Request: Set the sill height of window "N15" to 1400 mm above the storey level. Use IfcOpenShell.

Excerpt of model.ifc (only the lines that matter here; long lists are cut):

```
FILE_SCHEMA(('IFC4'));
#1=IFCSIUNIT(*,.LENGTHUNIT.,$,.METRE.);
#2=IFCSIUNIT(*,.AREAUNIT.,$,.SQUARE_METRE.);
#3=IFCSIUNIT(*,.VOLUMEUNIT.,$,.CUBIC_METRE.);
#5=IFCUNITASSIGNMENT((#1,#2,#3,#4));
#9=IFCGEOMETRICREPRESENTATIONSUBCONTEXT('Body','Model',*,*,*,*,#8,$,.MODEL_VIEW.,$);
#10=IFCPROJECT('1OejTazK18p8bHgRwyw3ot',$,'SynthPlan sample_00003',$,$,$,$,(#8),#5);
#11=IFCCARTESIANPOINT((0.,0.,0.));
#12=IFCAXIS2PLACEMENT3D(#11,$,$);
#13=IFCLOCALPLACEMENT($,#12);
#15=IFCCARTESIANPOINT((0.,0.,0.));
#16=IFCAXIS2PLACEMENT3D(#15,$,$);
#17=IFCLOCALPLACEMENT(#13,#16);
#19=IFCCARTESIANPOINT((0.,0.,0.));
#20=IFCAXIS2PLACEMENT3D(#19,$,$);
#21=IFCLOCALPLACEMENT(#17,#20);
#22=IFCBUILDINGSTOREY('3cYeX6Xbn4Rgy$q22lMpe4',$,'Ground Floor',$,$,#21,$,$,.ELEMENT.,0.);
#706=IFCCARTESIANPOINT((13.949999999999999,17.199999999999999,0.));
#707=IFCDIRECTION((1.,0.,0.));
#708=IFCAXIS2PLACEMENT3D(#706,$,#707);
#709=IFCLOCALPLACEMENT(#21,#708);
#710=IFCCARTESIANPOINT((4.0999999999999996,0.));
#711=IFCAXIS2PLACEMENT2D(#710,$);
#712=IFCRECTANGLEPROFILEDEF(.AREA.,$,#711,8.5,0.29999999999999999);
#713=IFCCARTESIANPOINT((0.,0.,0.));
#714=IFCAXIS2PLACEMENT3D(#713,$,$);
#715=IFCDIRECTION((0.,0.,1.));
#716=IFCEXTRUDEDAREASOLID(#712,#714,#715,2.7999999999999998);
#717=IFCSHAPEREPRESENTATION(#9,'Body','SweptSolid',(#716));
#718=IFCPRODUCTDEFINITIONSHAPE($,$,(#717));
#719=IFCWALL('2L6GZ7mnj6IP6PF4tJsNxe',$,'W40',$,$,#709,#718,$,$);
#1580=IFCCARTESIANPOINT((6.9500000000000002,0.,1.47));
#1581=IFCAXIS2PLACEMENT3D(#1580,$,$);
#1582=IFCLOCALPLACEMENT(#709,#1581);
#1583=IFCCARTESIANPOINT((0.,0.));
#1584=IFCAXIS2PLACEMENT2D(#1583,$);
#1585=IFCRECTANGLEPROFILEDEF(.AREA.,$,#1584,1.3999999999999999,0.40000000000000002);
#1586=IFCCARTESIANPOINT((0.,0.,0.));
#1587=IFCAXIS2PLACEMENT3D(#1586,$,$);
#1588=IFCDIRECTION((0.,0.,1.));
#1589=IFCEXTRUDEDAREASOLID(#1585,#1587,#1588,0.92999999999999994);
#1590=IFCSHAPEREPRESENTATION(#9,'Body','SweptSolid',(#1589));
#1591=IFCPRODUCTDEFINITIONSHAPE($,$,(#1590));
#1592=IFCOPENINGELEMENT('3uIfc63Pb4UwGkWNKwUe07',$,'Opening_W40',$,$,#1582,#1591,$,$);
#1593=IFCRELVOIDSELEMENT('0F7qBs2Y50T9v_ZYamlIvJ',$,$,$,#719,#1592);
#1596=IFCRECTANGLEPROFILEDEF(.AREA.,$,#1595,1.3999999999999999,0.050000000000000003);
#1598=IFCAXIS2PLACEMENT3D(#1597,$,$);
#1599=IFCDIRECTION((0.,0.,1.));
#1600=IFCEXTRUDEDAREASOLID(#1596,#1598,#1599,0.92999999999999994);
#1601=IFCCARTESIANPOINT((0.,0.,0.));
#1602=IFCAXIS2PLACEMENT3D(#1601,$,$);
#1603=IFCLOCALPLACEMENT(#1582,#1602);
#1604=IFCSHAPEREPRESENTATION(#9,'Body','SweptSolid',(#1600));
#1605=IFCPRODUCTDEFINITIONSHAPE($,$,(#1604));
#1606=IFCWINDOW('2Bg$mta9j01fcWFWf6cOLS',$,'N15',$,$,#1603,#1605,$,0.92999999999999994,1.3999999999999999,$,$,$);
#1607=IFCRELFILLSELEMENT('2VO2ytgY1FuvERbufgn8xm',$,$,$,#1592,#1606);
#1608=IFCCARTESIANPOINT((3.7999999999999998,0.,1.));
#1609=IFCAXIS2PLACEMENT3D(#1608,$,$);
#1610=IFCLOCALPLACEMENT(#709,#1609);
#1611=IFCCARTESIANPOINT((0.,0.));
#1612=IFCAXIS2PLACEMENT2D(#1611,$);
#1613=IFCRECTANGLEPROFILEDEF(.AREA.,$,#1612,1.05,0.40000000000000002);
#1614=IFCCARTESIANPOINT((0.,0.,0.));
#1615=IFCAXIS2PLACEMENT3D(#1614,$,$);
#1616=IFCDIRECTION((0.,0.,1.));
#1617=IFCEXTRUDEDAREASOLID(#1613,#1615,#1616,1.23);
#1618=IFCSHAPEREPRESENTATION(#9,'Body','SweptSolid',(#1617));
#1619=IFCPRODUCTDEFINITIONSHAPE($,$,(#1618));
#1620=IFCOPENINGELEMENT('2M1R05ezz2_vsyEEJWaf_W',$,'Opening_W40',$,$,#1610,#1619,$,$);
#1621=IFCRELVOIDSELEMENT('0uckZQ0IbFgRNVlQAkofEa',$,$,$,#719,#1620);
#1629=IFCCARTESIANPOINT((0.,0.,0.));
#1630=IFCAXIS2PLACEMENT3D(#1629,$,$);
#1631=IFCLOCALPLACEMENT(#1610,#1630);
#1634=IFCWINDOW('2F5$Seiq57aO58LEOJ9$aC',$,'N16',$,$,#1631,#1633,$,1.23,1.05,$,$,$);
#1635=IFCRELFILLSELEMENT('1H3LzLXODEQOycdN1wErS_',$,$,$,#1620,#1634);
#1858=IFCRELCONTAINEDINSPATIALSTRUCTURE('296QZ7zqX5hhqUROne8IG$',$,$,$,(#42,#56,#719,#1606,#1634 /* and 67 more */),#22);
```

```python
import numpy as np
import ifcopenshell
import ifcopenshell.api.geometry
import ifcopenshell.geom
import ifcopenshell.util.element
import ifcopenshell.util.placement
import ifcopenshell.util.shape
import ifcopenshell.util.unit

model = ifcopenshell.open("model.ifc")
unit_scale = ifcopenshell.util.unit.calculate_unit_scale(model)

window = model.by_id(1606)
opening = window.FillsVoids[0].RelatingOpeningElement
storey = ifcopenshell.util.element.get_container(window, ifc_class="IfcBuildingStorey")
level = ifcopenshell.util.placement.get_local_placement(storey.ObjectPlacement)[2, 3]

# The opening's origin need not be at the sill, so measure its lowest point.
shape = ifcopenshell.geom.create_shape(ifcopenshell.geom.settings(), opening)
bottom = ifcopenshell.util.shape.get_shape_bottom_elevation(shape, shape.geometry) / unit_scale
dz = level + 1.4 / unit_scale - bottom

shift = np.array([0.0, 0.0, dz])
# The window is placed relative to its opening, so it follows when the opening moves.
matrix = ifcopenshell.util.placement.get_local_placement(opening.ObjectPlacement)
matrix[:3, 3] += shift
ifcopenshell.api.geometry.edit_object_placement(
    model, product=opening, matrix=matrix, is_si=False, should_transform_children=True
)

print(f"moved by {dz * unit_scale:+.3f} m")

model.write("model_v2.ifc")
```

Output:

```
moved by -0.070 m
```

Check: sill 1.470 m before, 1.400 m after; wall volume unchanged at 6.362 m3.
